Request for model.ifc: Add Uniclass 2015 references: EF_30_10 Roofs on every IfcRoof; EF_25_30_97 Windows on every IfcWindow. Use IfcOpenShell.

First a look at what the model holds.

```python
import ifcopenshell

model = ifcopenshell.open("model.ifc")
print(model.schema)
print("classifications:", [c.Name for c in model.by_type("IfcClassification")])
for ifc_class in ("IfcDoor", "IfcRoof", "IfcStair", "IfcWall", "IfcWindow"):
    print(ifc_class, len(model.by_type(ifc_class)))
```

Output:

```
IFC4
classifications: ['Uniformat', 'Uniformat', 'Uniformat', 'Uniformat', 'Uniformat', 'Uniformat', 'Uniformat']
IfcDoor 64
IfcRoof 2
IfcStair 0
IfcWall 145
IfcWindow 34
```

```python
import ifcopenshell
import ifcopenshell.api.classification

model = ifcopenshell.open("model.ifc")

system = ifcopenshell.api.classification.add_classification(model, classification="Uniclass 2015")

codes = {
    "IfcRoof": ("EF_30_10", "Roofs"),
    "IfcWindow": ("EF_25_30_97", "Windows"),
}
for ifc_class, (code, name) in codes.items():
    products = model.by_type(ifc_class)
    ifcopenshell.api.classification.add_reference(
        model, products=products, classification=system, identification=code, name=name
    )
    print(code, len(products))

model.write("model_updated.ifc")
```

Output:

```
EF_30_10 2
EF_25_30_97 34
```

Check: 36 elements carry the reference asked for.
